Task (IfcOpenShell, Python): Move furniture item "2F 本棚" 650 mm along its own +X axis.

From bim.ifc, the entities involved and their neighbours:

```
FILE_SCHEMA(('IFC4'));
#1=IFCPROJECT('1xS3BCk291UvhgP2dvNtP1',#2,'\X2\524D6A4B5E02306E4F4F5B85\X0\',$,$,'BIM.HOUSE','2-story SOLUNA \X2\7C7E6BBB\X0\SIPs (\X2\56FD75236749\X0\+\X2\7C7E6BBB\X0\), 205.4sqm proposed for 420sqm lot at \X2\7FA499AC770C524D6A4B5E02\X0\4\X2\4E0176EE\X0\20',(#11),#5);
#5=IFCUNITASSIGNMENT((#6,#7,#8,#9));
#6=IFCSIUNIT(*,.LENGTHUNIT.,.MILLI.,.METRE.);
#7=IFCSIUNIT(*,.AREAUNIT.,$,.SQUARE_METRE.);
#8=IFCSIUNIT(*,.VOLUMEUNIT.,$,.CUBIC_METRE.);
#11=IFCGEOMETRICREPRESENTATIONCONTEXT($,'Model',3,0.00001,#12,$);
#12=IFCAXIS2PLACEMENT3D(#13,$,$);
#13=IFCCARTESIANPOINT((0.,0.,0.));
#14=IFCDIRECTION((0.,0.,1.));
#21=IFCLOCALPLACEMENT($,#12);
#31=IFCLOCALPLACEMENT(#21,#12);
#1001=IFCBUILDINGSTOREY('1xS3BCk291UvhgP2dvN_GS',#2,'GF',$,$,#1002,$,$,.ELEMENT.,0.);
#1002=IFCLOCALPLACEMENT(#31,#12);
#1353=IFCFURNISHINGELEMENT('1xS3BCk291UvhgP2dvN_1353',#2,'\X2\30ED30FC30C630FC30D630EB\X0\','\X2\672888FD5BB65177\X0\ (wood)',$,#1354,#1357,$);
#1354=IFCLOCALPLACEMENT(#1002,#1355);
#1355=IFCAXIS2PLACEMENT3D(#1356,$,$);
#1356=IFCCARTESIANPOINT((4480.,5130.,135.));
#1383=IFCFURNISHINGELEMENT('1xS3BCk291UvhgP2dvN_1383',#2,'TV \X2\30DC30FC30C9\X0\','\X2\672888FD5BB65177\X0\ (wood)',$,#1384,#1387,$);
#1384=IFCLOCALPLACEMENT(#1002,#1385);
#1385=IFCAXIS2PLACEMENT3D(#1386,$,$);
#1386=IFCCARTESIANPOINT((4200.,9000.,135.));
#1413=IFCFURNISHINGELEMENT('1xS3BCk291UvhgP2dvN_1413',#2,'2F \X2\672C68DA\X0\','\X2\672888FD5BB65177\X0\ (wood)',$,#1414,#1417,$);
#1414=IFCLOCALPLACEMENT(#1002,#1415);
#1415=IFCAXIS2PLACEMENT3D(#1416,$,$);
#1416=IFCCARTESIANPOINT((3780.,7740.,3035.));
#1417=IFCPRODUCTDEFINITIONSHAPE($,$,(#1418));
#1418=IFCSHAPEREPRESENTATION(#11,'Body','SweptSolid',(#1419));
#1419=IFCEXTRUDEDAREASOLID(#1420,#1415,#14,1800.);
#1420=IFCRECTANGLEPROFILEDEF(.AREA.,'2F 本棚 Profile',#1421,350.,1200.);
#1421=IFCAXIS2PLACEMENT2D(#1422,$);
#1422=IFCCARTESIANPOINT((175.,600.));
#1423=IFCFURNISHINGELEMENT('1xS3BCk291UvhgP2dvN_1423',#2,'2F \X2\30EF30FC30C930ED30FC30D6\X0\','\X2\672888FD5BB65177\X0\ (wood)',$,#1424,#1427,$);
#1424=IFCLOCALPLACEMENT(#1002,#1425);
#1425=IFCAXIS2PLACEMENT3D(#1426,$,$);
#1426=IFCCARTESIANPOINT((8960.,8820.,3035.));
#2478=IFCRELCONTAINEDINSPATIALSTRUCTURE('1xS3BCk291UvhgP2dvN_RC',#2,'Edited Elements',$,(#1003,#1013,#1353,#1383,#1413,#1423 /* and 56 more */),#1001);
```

```python
import ifcopenshell
import ifcopenshell.api.geometry
import ifcopenshell.util.placement
import ifcopenshell.util.unit

model = ifcopenshell.open("bim.ifc")
unit_scale = ifcopenshell.util.unit.calculate_unit_scale(model)

item = model.by_guid("1xS3BCk291UvhgP2dvN_1413")
matrix = ifcopenshell.util.placement.get_local_placement(item.ObjectPlacement)
matrix[:3, 3] += matrix[:3, 0] * 0.65 / unit_scale
ifcopenshell.api.geometry.edit_object_placement(model, product=item, matrix=matrix, is_si=False)

print(ifcopenshell.util.placement.get_local_placement(item.ObjectPlacement).round(3) + 0.0)

model.write("bim_v2.ifc")
```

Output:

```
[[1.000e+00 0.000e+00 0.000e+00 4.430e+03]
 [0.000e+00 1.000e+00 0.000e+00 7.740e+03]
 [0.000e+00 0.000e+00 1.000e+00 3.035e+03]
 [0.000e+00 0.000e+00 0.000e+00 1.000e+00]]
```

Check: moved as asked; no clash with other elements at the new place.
